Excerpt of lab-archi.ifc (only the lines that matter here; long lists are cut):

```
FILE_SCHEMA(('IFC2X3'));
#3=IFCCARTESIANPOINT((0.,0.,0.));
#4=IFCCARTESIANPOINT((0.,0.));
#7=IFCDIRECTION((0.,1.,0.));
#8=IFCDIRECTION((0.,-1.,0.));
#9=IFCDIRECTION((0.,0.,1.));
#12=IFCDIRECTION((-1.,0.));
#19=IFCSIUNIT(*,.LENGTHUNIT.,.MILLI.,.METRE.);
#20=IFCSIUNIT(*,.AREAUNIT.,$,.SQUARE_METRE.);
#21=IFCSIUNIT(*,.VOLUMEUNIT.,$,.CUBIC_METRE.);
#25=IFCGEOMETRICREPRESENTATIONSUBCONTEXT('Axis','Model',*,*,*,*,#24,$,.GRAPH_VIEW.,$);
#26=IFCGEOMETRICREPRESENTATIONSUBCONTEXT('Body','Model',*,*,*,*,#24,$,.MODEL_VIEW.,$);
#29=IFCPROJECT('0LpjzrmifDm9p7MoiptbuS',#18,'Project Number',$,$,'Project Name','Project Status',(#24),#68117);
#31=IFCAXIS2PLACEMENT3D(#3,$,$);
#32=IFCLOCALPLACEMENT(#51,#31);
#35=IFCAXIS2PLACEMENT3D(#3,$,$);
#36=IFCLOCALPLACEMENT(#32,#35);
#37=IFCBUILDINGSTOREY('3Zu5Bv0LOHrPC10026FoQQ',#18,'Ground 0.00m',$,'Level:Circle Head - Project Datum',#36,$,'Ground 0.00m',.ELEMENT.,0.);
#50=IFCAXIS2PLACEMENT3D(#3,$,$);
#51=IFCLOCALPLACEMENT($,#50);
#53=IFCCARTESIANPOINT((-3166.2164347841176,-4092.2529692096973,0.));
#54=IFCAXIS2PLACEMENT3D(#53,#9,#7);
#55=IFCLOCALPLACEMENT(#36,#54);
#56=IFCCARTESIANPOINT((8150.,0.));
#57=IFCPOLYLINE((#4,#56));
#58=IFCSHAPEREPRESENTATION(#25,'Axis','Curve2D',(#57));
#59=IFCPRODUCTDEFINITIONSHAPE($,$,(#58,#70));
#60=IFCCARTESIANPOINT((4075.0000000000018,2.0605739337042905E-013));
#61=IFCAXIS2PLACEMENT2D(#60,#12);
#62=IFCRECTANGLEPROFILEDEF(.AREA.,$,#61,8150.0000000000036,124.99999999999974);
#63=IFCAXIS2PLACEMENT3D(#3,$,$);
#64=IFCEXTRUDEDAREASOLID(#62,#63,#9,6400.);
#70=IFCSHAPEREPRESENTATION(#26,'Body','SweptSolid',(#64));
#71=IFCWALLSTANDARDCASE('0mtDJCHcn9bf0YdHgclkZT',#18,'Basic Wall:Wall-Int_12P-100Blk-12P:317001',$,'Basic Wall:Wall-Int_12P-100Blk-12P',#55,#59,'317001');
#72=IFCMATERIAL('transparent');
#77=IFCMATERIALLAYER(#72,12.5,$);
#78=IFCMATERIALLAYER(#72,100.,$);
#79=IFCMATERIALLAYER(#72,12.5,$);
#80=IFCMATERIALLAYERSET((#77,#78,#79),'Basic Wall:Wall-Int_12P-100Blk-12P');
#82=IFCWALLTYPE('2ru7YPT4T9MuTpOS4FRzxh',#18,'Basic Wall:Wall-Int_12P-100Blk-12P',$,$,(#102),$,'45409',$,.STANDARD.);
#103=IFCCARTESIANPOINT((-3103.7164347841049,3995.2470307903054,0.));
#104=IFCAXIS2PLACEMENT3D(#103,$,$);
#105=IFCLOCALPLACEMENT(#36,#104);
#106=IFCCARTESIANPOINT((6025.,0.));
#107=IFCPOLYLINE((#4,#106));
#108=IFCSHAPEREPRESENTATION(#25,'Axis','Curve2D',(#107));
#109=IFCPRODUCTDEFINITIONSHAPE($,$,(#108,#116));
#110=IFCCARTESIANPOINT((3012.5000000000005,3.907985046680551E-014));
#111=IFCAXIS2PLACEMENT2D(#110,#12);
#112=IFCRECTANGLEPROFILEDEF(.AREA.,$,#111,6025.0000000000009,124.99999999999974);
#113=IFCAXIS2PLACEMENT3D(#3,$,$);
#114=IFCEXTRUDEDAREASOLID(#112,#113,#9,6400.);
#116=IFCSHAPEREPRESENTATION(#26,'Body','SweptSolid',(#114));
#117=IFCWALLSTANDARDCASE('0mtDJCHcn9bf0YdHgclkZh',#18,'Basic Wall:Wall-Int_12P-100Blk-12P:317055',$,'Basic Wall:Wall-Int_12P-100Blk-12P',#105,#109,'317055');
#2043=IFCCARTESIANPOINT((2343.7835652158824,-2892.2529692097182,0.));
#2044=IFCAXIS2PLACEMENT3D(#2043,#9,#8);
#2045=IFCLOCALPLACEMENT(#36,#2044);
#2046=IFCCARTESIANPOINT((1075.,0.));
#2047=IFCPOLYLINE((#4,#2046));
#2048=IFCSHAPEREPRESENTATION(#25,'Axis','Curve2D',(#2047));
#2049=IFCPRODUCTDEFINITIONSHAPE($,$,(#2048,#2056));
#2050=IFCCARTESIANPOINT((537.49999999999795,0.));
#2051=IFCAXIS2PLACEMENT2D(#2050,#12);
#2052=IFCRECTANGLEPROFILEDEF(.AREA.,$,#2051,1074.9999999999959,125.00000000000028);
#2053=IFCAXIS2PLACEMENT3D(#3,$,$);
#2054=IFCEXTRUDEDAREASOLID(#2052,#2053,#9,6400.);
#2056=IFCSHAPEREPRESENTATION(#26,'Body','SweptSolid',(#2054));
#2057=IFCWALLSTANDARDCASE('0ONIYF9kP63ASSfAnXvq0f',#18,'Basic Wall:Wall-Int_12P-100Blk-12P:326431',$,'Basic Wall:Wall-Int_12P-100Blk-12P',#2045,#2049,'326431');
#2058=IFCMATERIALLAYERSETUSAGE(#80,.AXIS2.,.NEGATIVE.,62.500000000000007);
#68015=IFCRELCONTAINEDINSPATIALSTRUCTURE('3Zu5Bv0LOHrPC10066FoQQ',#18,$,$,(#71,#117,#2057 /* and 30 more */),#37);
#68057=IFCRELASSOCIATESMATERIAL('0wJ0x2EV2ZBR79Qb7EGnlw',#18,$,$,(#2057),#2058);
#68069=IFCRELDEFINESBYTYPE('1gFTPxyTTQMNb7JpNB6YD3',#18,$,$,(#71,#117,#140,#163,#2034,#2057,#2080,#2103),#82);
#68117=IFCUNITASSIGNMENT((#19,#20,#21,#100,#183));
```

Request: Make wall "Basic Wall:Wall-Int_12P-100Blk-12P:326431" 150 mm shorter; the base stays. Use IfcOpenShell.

```python
import ifcopenshell
import ifcopenshell.geom
import ifcopenshell.util.representation
import ifcopenshell.util.shape
import ifcopenshell.util.unit

model = ifcopenshell.open("lab-archi.ifc")
unit_scale = ifcopenshell.util.unit.calculate_unit_scale(model)
settings = ifcopenshell.geom.settings()


def volume(element):
    """Net volume in cubic metres, openings subtracted."""
    shape = ifcopenshell.geom.create_shape(settings, element)
    return ifcopenshell.util.shape.get_volume(shape.geometry)


wall = model.by_id(2057)
before = volume(wall)

body = ifcopenshell.util.representation.get_representation(wall, "Model", "Body")
solid = body.Items[0]
old_height = solid.Depth
solid.Depth -= 0.15 / unit_scale
after = volume(wall)

print(f"height {old_height:g} -> {solid.Depth:g}, volume {before:.3f} -> {after:.3f} m3")

model.write("lab-archi_rev.ifc")
```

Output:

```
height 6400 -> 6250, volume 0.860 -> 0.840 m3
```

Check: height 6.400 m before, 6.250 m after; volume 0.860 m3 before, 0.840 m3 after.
